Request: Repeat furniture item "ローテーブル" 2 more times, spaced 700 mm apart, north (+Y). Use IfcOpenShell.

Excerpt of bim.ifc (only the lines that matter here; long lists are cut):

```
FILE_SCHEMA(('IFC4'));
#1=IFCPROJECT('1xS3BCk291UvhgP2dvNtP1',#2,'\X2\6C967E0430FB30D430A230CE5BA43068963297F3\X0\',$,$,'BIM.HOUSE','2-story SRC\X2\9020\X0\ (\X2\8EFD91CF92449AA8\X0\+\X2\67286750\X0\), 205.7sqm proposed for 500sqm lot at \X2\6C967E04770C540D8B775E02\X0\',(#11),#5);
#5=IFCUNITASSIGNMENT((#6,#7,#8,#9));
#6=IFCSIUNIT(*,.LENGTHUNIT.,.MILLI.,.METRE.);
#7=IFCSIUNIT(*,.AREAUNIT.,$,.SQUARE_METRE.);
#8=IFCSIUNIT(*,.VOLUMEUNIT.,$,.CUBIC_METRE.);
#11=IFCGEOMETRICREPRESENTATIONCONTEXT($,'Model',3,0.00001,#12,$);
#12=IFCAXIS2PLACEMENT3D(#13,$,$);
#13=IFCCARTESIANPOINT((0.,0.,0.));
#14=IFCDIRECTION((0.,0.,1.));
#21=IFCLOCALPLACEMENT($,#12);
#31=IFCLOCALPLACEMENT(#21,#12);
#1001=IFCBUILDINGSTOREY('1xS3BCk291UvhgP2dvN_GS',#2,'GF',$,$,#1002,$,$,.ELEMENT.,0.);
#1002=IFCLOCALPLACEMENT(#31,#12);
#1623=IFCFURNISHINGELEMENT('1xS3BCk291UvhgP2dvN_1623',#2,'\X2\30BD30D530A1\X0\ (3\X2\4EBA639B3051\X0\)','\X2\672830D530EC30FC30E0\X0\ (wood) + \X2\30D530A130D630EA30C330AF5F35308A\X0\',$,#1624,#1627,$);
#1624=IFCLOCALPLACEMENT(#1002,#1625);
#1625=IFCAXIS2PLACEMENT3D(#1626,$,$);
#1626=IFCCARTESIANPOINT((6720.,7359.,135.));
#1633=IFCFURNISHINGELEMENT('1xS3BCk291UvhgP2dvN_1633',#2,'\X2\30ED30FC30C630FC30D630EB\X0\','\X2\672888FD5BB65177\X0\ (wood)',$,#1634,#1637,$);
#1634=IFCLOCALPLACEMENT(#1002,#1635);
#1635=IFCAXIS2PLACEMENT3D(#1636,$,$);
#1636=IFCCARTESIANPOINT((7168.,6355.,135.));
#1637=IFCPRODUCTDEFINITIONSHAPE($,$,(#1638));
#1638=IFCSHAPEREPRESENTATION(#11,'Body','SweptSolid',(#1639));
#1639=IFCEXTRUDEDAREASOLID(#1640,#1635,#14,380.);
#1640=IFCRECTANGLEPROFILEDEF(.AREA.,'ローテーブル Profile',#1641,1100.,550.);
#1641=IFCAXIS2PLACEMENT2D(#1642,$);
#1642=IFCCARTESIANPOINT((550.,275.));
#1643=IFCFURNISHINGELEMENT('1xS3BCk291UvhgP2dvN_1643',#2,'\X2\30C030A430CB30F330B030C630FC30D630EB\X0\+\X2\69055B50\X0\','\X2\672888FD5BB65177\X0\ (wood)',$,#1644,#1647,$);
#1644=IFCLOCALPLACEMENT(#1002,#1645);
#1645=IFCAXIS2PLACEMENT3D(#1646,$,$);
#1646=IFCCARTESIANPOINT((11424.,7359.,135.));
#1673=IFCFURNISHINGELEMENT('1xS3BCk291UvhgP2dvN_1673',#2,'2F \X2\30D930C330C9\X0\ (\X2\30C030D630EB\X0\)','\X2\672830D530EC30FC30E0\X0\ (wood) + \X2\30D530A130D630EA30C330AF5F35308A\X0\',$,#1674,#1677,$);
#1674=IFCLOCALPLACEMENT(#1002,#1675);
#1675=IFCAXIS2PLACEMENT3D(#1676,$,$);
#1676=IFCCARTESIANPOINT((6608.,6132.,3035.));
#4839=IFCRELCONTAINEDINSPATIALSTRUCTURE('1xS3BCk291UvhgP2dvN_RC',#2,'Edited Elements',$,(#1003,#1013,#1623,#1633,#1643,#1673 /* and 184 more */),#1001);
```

```python
import numpy as np
import ifcopenshell
import ifcopenshell.api.geometry
import ifcopenshell.api.root
import ifcopenshell.util.element
import ifcopenshell.util.placement
import ifcopenshell.util.unit

model = ifcopenshell.open("bim.ifc")
unit_scale = ifcopenshell.util.unit.calculate_unit_scale(model)


def reuse_history(source, copy):
    """copy_class also copies each property set's owner history, people and application; keep the originals."""
    for rel in copy.IsDefinedBy:
        if rel.is_a("IfcRelDefinesByProperties") and (history := rel.RelatingPropertyDefinition.OwnerHistory):
            rel.RelatingPropertyDefinition.OwnerHistory = source.OwnerHistory
            ifcopenshell.util.element.remove_deep2(model, history)


source = model.by_guid("1xS3BCk291UvhgP2dvN_1633")
base = ifcopenshell.util.placement.get_local_placement(source.ObjectPlacement)
step = np.array([0.0, 1.0, 0.0]) * 0.7 / unit_scale

for i in range(1, 3):
    copy = ifcopenshell.api.root.copy_class(model, product=source)
    copy.Representation = ifcopenshell.util.element.copy_deep(
        model, source.Representation, exclude=["IfcGeometricRepresentationContext", "IfcRepresentationMap"]
    )
    reuse_history(source, copy)
    matrix = base.copy()
    matrix[:3, 3] += i * step
    print("added at", matrix[:3, 3].round(3) + 0.0)
    ifcopenshell.api.geometry.edit_object_placement(model, product=copy, matrix=matrix, is_si=False)

model.write("bim_rev.ifc")
```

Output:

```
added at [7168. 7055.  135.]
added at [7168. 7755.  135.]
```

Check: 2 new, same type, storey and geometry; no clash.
